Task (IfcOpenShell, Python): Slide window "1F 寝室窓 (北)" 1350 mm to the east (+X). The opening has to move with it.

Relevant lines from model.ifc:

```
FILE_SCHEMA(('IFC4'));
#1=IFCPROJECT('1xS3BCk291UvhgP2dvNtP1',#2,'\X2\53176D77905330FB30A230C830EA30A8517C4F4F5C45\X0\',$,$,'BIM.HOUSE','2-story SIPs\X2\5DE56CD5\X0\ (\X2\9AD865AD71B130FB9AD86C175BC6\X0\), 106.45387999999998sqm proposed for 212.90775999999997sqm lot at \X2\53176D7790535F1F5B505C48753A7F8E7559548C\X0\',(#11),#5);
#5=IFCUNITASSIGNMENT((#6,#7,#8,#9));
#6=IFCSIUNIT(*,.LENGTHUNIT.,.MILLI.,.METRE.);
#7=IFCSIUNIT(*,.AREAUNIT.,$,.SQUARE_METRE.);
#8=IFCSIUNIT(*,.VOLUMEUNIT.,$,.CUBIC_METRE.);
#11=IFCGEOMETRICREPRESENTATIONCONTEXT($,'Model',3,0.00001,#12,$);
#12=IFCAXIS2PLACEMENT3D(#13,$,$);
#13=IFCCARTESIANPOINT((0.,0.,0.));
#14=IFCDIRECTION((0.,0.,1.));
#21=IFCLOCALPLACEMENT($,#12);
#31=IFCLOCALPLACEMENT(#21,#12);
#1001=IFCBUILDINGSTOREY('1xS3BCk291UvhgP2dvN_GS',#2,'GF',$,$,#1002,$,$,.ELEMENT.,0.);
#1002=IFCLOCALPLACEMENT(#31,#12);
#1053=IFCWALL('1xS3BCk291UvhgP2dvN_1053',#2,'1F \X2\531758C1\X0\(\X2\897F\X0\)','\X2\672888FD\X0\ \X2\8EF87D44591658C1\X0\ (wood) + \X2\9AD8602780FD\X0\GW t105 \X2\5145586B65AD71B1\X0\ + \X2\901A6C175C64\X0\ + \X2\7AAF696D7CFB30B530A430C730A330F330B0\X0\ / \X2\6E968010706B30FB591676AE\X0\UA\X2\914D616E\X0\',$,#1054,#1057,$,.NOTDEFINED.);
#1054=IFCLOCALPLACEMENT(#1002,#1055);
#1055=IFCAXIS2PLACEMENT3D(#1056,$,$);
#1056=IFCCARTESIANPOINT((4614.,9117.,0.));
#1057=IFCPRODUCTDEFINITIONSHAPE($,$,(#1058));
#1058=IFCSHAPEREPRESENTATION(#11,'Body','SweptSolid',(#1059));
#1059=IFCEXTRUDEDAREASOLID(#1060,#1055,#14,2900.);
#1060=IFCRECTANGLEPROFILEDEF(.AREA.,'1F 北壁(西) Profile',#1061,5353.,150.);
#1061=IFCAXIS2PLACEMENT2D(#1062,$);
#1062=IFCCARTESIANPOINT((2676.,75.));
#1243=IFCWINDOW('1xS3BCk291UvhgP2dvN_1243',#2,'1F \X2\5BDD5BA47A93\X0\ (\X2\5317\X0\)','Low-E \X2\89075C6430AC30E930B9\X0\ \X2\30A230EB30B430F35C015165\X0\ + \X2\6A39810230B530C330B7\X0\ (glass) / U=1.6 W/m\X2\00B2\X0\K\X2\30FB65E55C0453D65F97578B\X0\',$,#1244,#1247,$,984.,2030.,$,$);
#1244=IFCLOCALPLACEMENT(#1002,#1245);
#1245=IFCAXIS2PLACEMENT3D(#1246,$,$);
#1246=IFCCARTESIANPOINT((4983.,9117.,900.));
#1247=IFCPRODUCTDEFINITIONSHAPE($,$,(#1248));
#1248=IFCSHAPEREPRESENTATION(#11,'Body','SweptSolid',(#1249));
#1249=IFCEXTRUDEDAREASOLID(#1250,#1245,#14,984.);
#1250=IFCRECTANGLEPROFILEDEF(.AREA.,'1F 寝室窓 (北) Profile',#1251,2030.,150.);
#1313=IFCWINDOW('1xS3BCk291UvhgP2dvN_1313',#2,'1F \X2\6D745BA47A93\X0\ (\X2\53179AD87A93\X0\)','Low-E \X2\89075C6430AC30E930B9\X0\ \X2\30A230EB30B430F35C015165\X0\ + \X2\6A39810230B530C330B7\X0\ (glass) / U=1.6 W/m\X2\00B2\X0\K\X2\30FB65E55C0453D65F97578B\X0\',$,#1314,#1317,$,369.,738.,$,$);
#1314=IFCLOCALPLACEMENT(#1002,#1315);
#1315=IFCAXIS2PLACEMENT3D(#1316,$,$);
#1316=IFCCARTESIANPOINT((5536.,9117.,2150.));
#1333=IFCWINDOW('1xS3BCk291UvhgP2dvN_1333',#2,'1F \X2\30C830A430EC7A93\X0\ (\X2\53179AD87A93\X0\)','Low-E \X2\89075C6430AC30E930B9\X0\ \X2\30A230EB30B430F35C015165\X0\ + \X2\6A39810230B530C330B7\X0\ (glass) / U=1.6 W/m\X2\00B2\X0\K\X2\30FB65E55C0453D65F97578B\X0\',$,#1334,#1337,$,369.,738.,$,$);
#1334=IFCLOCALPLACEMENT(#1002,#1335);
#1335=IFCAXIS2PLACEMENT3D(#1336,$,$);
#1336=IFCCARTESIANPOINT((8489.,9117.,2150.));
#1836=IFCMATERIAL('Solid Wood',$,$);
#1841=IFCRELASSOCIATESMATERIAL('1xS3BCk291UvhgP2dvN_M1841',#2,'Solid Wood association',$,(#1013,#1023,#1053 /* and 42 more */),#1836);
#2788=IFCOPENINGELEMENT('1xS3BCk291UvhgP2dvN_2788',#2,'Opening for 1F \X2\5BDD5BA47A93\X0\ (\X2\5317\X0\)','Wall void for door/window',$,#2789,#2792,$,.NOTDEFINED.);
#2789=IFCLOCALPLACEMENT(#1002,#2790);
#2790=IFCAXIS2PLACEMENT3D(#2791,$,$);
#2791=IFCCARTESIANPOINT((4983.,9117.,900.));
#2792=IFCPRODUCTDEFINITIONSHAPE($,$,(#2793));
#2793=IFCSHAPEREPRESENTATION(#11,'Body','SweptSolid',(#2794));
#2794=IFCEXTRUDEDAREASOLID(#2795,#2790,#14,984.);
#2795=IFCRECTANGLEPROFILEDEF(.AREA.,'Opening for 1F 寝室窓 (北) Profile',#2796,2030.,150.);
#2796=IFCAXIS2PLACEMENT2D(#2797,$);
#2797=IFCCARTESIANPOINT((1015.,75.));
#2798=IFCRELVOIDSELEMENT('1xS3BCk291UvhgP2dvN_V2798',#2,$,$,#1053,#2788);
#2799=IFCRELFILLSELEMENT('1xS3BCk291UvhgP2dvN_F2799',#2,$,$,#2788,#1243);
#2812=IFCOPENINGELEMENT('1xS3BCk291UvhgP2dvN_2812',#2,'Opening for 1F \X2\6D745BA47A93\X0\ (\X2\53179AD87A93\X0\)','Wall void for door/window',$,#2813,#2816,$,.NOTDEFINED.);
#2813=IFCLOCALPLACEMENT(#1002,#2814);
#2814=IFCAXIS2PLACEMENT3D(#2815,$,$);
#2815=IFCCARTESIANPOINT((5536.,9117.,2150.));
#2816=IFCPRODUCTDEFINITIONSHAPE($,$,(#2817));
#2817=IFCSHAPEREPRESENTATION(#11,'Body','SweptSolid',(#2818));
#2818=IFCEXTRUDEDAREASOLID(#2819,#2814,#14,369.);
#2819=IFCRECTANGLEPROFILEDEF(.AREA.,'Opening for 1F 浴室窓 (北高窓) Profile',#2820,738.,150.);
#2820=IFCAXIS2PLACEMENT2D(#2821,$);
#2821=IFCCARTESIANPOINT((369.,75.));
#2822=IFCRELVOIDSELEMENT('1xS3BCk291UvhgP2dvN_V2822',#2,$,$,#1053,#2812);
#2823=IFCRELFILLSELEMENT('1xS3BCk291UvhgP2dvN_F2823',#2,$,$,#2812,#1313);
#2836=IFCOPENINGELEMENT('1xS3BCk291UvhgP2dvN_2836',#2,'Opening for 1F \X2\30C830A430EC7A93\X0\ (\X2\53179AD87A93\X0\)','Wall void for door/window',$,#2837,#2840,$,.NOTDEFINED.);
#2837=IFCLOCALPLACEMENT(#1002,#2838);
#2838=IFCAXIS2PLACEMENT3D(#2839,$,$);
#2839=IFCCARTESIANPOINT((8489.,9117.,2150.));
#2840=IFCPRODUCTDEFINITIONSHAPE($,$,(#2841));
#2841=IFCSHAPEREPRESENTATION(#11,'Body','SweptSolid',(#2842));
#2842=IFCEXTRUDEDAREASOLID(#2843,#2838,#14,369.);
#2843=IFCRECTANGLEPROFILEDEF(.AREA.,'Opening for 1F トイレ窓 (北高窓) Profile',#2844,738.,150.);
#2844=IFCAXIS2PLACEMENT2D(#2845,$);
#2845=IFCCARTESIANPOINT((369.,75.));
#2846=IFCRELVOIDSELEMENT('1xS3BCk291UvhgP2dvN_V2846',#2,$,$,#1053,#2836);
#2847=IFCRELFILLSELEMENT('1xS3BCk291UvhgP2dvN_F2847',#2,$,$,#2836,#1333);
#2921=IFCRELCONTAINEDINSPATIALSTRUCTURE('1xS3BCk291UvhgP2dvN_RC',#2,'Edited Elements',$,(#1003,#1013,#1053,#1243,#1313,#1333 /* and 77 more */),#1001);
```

```python
import ifcopenshell
import ifcopenshell.api.geometry
import ifcopenshell.util.placement

model = ifcopenshell.open("model.ifc")

window = model.by_id(1243)
opening = window.FillsVoids[0].RelatingOpeningElement
wall = opening.VoidsElements[0].RelatingBuildingElement

wall_matrix = ifcopenshell.util.placement.get_local_placement(wall.ObjectPlacement)
shift = wall_matrix[:3, 0] * 1350.0
before = ifcopenshell.util.placement.get_local_placement(window.ObjectPlacement)[:3, 3].copy()

# The window is not placed relative to its opening, so move both.
for product in (opening, window):
    matrix = ifcopenshell.util.placement.get_local_placement(product.ObjectPlacement)
    matrix[:3, 3] += shift
    ifcopenshell.api.geometry.edit_object_placement(model, product=product, matrix=matrix, is_si=False)

after = ifcopenshell.util.placement.get_local_placement(window.ObjectPlacement)[:3, 3]
print("window moved by", (after - before).round(3) + 0.0)

model.write("model_updated.ifc")
```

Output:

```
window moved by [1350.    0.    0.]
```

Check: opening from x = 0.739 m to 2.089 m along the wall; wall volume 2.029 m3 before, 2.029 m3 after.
